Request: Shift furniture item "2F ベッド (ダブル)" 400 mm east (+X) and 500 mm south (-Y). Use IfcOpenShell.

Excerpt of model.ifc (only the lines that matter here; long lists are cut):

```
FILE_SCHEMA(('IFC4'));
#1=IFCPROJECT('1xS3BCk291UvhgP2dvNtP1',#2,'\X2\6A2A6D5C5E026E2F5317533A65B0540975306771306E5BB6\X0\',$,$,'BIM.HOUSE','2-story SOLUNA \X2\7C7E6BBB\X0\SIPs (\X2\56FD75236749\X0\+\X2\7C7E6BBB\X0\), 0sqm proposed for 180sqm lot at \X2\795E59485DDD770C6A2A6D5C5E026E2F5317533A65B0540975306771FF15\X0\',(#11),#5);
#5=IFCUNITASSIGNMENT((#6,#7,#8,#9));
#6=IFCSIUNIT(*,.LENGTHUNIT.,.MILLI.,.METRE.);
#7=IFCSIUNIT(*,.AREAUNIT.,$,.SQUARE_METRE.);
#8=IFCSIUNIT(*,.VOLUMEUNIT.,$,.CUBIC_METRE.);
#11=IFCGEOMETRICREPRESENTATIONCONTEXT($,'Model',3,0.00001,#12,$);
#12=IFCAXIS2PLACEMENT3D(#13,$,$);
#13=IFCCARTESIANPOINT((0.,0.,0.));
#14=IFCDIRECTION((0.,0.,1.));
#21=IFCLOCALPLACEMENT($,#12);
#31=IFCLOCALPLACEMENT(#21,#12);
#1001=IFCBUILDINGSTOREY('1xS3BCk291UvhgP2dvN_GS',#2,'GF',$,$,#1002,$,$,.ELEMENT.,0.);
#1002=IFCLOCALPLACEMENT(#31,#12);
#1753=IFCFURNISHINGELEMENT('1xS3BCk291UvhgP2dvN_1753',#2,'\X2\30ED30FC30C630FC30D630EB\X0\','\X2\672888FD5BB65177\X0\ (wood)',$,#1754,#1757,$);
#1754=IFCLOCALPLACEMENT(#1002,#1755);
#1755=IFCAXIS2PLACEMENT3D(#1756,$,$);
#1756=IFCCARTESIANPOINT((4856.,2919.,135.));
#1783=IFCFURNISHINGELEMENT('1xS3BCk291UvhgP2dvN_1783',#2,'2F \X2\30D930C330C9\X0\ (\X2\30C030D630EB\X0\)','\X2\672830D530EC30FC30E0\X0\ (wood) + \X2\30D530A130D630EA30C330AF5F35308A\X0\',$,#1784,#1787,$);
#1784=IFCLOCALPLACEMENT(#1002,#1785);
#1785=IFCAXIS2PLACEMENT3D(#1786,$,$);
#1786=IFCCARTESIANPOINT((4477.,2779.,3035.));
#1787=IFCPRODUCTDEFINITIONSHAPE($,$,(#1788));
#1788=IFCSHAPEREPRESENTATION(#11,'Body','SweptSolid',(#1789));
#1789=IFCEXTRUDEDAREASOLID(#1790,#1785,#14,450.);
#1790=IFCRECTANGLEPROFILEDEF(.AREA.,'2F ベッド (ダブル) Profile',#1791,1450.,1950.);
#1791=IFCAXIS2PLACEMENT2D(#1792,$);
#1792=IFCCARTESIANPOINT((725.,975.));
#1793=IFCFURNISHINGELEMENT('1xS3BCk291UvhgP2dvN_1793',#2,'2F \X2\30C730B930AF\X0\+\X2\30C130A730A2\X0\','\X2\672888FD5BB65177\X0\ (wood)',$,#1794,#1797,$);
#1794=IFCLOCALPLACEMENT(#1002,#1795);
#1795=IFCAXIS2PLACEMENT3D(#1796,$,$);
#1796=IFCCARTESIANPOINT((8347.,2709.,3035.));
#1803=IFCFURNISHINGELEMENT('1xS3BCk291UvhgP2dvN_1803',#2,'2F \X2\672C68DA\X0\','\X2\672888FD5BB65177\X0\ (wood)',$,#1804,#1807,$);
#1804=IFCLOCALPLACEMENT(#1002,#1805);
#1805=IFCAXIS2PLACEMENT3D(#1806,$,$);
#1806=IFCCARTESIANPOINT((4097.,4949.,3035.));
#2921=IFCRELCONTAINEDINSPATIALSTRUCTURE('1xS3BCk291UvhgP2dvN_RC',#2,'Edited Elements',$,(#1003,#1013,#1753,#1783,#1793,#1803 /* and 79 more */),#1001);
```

```python
import ifcopenshell
import ifcopenshell.api.geometry
import ifcopenshell.util.placement
import ifcopenshell.util.unit

model = ifcopenshell.open("model.ifc")
unit_scale = ifcopenshell.util.unit.calculate_unit_scale(model)

item = model.by_guid("1xS3BCk291UvhgP2dvN_1783")
matrix = ifcopenshell.util.placement.get_local_placement(item.ObjectPlacement)
matrix[0, 3] += 0.4 / unit_scale
matrix[1, 3] -= 0.5 / unit_scale
ifcopenshell.api.geometry.edit_object_placement(model, product=item, matrix=matrix, is_si=False)

print(ifcopenshell.util.placement.get_local_placement(item.ObjectPlacement).round(3) + 0.0)

model.write("model_edited.ifc")
```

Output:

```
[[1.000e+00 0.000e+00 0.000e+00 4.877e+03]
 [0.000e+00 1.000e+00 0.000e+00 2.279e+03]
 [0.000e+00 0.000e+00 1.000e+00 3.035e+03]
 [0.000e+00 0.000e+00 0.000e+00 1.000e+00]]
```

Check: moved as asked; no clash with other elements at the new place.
